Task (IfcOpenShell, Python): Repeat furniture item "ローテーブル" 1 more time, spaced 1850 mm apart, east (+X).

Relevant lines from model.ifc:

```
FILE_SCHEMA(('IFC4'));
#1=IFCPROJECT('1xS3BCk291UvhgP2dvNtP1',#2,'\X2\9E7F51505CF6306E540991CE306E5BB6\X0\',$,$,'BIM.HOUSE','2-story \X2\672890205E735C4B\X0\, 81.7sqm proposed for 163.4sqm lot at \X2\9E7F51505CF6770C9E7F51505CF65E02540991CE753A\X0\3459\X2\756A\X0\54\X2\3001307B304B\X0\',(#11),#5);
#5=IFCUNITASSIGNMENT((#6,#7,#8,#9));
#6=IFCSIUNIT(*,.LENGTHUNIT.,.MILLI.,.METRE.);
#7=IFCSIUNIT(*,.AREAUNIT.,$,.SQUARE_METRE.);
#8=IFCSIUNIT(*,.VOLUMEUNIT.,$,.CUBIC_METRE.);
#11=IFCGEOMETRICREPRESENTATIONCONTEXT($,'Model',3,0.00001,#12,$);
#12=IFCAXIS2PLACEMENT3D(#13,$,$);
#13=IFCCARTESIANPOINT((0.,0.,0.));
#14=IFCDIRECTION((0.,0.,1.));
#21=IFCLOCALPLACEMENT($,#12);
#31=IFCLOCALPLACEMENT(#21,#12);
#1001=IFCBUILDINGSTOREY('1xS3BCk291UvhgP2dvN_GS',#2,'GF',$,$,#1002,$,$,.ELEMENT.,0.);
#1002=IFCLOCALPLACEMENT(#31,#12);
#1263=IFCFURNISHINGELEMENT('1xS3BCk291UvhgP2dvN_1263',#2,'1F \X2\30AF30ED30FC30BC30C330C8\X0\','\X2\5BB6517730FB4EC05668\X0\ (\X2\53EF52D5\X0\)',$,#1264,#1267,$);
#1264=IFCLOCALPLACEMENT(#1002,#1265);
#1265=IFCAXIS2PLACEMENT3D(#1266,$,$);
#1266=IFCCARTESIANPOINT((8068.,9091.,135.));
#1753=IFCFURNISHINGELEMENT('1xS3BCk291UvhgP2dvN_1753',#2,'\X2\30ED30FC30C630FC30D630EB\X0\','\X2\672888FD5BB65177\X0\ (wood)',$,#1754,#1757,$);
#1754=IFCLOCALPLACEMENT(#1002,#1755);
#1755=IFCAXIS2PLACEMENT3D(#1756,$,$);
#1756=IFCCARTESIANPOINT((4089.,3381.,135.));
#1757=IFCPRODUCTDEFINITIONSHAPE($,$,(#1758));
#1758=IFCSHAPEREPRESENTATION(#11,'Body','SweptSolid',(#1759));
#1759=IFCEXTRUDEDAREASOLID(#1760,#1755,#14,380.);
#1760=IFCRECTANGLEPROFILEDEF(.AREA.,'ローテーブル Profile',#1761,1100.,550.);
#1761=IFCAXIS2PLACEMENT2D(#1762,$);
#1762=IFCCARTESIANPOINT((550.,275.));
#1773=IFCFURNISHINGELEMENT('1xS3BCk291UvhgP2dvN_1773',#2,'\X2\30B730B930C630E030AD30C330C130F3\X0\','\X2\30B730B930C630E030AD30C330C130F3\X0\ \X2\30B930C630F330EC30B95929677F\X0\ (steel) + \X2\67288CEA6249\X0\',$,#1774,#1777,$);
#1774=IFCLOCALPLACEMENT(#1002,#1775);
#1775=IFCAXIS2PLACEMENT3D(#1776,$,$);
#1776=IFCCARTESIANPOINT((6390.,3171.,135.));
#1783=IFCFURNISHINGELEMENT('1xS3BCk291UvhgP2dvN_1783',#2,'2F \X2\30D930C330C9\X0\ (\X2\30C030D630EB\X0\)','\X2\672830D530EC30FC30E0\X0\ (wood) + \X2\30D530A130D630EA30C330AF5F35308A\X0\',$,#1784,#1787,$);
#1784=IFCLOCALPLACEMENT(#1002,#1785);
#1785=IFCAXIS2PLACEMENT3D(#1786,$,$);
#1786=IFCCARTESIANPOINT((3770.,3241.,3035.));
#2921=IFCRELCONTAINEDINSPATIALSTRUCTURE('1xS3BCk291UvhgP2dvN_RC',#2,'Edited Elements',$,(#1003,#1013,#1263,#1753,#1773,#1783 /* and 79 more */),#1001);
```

```python
import numpy as np
import ifcopenshell
import ifcopenshell.api.geometry
import ifcopenshell.api.root
import ifcopenshell.util.element
import ifcopenshell.util.placement

model = ifcopenshell.open("model.ifc")


def reuse_history(source, copy):
    """copy_class also copies each property set's owner history, people and application; keep the originals."""
    for rel in copy.IsDefinedBy:
        if rel.is_a("IfcRelDefinesByProperties") and (history := rel.RelatingPropertyDefinition.OwnerHistory):
            rel.RelatingPropertyDefinition.OwnerHistory = source.OwnerHistory
            ifcopenshell.util.element.remove_deep2(model, history)


source = model.by_guid("1xS3BCk291UvhgP2dvN_1753")
base = ifcopenshell.util.placement.get_local_placement(source.ObjectPlacement)
step = np.array([1.0, 0.0, 0.0]) * 1850.0

for i in range(1, 2):
    copy = ifcopenshell.api.root.copy_class(model, product=source)
    copy.Representation = ifcopenshell.util.element.copy_deep(
        model, source.Representation, exclude=["IfcGeometricRepresentationContext", "IfcRepresentationMap"]
    )
    reuse_history(source, copy)
    matrix = base.copy()
    matrix[:3, 3] += i * step
    print("added at", matrix[:3, 3].round(3) + 0.0)
    ifcopenshell.api.geometry.edit_object_placement(model, product=copy, matrix=matrix, is_si=False)

model.write("model-out.ifc")
```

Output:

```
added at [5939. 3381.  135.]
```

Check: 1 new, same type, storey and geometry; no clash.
